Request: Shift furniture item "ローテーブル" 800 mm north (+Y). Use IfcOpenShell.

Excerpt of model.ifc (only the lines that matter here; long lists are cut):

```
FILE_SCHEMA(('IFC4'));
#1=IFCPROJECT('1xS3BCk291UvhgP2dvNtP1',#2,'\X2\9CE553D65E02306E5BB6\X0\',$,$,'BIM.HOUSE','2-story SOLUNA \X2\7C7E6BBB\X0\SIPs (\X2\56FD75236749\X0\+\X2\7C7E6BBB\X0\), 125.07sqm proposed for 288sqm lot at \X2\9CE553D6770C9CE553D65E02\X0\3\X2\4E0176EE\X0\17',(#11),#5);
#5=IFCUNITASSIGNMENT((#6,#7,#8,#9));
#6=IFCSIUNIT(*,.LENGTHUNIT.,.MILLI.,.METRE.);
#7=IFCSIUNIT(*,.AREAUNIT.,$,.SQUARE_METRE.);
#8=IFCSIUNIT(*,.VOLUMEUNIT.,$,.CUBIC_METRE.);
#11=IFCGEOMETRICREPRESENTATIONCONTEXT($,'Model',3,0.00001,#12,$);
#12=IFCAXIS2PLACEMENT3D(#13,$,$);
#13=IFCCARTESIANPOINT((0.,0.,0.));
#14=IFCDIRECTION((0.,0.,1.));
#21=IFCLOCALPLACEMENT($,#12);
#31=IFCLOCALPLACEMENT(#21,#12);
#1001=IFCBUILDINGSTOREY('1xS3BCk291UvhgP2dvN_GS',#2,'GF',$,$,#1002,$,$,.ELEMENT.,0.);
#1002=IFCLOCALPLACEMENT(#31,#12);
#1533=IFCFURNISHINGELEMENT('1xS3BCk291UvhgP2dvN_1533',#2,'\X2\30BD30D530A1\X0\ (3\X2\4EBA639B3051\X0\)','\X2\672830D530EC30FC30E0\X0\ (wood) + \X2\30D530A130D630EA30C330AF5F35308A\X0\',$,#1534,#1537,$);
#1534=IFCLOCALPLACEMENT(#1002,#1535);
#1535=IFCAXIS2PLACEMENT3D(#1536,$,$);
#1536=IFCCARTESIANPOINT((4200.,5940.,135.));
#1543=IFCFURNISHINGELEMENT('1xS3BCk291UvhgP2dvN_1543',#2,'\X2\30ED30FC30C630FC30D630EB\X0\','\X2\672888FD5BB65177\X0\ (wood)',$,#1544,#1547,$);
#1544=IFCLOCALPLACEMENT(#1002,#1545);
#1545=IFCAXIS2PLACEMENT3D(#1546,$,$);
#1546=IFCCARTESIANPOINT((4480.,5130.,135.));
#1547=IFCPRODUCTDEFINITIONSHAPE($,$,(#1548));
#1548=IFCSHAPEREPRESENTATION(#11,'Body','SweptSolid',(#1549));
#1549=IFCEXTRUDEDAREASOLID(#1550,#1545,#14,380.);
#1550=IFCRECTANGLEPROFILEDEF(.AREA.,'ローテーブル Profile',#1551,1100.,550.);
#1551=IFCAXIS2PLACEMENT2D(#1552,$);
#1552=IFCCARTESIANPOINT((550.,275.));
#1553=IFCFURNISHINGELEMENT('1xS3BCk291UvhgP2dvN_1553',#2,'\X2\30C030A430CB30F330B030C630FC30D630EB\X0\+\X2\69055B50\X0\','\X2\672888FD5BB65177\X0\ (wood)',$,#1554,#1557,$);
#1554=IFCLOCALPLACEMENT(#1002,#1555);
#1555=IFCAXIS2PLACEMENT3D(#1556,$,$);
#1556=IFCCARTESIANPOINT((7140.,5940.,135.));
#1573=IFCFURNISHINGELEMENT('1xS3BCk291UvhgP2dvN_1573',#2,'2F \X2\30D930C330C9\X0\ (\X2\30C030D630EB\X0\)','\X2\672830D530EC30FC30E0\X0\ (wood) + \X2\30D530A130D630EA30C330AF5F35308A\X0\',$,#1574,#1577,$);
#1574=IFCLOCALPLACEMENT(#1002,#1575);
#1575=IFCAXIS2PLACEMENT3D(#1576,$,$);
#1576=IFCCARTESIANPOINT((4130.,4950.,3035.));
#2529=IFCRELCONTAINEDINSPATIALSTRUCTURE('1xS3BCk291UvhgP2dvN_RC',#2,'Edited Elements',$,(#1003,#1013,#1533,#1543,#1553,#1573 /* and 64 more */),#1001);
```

```python
import ifcopenshell
import ifcopenshell.api.geometry
import ifcopenshell.util.placement
import ifcopenshell.util.unit

model = ifcopenshell.open("model.ifc")
unit_scale = ifcopenshell.util.unit.calculate_unit_scale(model)

item = model.by_guid("1xS3BCk291UvhgP2dvN_1543")
matrix = ifcopenshell.util.placement.get_local_placement(item.ObjectPlacement)
matrix[1, 3] += 0.8 / unit_scale
ifcopenshell.api.geometry.edit_object_placement(model, product=item, matrix=matrix, is_si=False)

print(ifcopenshell.util.placement.get_local_placement(item.ObjectPlacement).round(3) + 0.0)

model.write("model_rev.ifc")
```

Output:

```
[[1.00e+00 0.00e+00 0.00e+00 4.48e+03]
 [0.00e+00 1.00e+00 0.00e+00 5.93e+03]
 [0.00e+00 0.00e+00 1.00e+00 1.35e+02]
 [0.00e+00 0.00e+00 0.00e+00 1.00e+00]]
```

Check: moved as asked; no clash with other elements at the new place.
